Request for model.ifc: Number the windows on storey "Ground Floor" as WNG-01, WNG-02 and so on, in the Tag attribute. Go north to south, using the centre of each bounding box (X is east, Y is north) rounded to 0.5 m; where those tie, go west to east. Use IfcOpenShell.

First a look at what the model holds.

```python
import ifcopenshell
import ifcopenshell.util.element
import ifcopenshell.util.placement

model = ifcopenshell.open("model.ifc")
print(model.schema)
storey = next(s for s in model.by_type("IfcBuildingStorey") if s.Name == "Ground Floor")
windows = [e for e in ifcopenshell.util.element.get_decomposition(storey) if e.is_a("IfcWindow")]
for e in sorted(windows, key=lambda e: e.id()):
    origin = ifcopenshell.util.placement.get_local_placement(e.ObjectPlacement)[:3, 3]
    print(e.id(), e.Tag, e.Name, origin.round(2) + 0.0, sep=" | ")
```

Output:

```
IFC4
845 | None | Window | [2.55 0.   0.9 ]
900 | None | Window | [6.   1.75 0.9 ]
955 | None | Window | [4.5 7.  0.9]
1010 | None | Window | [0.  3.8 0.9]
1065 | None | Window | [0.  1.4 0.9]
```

```python
import ifcopenshell
import ifcopenshell.geom
import ifcopenshell.util.element
import ifcopenshell.util.shape

model = ifcopenshell.open("model.ifc")
settings = ifcopenshell.geom.settings()
settings.set("use-world-coords", True)


def centre(element):
    shape = ifcopenshell.geom.create_shape(settings, element)
    return ifcopenshell.util.shape.get_bbox_centroid(shape.geometry)


storey = next(s for s in model.by_type("IfcBuildingStorey") if s.Name == "Ground Floor")
windows = [e for e in ifcopenshell.util.element.get_decomposition(storey) if e.is_a("IfcWindow")]

# Insertion points can sit at a corner or the storey origin, so sort by the geometry (in metres).
centres = {e: centre(e) for e in windows}
windows.sort(key=lambda e: (-round(centres[e][1] / 0.5), centres[e][0]))

for i, e in enumerate(windows, start=1):
    number = f"WNG-{i:02d}"
    e.Tag = number
    print(e.id(), number)

model.write("model_updated.ifc")
```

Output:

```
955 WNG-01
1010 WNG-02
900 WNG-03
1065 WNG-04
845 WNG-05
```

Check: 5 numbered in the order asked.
